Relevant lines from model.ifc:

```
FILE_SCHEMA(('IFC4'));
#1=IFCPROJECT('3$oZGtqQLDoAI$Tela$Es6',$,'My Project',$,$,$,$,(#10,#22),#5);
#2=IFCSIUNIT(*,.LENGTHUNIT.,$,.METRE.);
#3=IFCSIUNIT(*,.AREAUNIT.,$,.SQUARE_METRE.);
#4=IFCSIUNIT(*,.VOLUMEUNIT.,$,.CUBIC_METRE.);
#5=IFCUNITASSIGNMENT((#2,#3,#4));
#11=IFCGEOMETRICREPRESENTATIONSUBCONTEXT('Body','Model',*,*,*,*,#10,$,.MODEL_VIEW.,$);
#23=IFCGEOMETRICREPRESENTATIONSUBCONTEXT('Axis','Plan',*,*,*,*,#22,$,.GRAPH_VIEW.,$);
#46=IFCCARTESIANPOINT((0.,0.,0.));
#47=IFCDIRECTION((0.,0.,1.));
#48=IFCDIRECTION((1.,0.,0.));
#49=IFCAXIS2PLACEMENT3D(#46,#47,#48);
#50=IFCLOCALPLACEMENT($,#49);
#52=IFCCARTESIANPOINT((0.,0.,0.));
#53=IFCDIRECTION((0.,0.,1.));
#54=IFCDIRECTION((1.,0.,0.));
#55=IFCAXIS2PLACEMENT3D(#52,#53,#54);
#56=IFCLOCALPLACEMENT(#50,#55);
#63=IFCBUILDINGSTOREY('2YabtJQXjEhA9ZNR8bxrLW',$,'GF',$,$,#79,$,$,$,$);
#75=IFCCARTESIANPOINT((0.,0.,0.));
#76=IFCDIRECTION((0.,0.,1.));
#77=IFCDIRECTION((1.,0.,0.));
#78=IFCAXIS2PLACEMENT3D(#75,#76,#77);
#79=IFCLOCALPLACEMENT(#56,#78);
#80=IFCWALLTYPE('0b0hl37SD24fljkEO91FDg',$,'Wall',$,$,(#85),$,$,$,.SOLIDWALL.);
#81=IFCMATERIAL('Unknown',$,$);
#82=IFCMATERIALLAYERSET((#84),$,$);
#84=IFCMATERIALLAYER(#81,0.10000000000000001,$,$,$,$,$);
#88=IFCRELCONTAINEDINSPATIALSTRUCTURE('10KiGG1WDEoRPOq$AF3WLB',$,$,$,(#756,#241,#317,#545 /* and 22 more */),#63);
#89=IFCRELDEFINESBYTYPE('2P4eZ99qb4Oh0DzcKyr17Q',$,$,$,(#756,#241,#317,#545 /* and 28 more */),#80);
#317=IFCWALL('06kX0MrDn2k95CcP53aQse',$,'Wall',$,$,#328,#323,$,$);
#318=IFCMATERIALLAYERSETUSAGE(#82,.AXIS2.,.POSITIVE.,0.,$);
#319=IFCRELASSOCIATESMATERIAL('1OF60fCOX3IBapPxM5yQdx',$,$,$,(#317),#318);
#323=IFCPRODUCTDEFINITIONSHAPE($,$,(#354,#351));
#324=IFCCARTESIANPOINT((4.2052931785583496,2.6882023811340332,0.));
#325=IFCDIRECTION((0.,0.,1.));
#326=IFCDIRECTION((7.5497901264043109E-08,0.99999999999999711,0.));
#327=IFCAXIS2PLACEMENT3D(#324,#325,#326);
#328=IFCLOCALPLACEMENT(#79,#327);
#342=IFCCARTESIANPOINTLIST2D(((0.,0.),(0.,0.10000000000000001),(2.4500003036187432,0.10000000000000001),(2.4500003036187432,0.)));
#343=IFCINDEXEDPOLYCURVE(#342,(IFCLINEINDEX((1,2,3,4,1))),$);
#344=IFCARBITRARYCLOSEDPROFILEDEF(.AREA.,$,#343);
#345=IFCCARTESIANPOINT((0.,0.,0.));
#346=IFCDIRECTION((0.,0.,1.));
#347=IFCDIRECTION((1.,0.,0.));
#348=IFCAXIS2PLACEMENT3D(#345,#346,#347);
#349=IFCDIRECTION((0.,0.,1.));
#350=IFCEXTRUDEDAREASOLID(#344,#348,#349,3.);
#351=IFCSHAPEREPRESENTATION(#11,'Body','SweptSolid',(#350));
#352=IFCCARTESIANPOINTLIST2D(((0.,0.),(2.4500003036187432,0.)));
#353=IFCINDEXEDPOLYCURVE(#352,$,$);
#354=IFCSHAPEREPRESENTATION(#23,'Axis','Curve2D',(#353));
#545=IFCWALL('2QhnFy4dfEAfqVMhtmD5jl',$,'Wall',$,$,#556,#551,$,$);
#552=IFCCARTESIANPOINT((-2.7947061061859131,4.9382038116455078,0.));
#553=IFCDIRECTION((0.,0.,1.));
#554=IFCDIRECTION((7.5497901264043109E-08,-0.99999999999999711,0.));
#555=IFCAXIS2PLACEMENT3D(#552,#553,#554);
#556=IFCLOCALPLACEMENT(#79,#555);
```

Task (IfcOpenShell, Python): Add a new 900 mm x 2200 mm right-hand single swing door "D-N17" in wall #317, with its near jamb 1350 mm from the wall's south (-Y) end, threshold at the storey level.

```python
import numpy as np
import ifcopenshell
import ifcopenshell.api.feature
import ifcopenshell.api.geometry
import ifcopenshell.api.root
import ifcopenshell.api.spatial
import ifcopenshell.geom
import ifcopenshell.util.element
import ifcopenshell.util.placement
import ifcopenshell.util.representation
import ifcopenshell.util.shape
import ifcopenshell.util.unit

model = ifcopenshell.open("model.ifc")
unit_scale = ifcopenshell.util.unit.calculate_unit_scale(model)
settings = ifcopenshell.geom.settings()


def volume(element):
    """Net volume in cubic metres, openings subtracted."""
    shape = ifcopenshell.geom.create_shape(settings, element)
    return ifcopenshell.util.shape.get_volume(shape.geometry)


wall = model.by_guid("06kX0MrDn2k95CcP53aQse")
storey = ifcopenshell.util.element.get_container(wall, ifc_class="IfcBuildingStorey")
context = ifcopenshell.util.representation.get_context(model, "Model", "Body", "MODEL_VIEW")
before = volume(wall)

width, height, from_end, sill = 0.9, 2.2, 1.35, 0.0  # metres

# The wall runs along its own X axis, and the end named is its -X end.
wall_shape = ifcopenshell.geom.create_shape(settings, wall)
x, y, z = ifcopenshell.util.shape.get_vertices(wall_shape.geometry).T
start = x.min() + from_end
face, thickness = float(y.min()), float(y.max() - y.min())
wall_matrix = ifcopenshell.util.placement.get_local_placement(wall.ObjectPlacement)
level = ifcopenshell.util.placement.get_local_placement(storey.ObjectPlacement)[2, 3]


def in_wall(x, y):
    """Placement at x, y metres in the wall's axes, at sill height."""
    matrix = wall_matrix.copy()
    matrix[:, 3] = wall_matrix @ np.array([x / unit_scale, y / unit_scale, 0.0, 1.0])
    matrix[2, 3] = level + sill / unit_scale
    return matrix


# Opening: a box that overshoots both wall faces by 50 mm.
opening = ifcopenshell.api.root.create_entity(model, ifc_class="IfcOpeningElement", predefined_type="OPENING")
box = ifcopenshell.api.geometry.add_wall_representation(
    model, context=context, length=width, height=height, thickness=thickness + 0.1
)
ifcopenshell.api.geometry.assign_representation(model, product=opening, representation=box)
ifcopenshell.api.geometry.edit_object_placement(model, product=opening, matrix=in_wall(start, face - 0.05), is_si=False)
ifcopenshell.api.feature.add_feature(model, feature=opening, element=wall)

door = ifcopenshell.api.root.create_entity(model, ifc_class="IfcDoor", name="D-N17", predefined_type="DOOR")
door.OverallWidth, door.OverallHeight = width / unit_scale, height / unit_scale
door.OperationType = "SINGLE_SWING_RIGHT"
body = ifcopenshell.api.geometry.add_door_representation(
    model,
    context=context,
    overall_width=door.OverallWidth,
    overall_height=door.OverallHeight,
    operation_type="SINGLE_SWING_RIGHT",
    lining_properties={"LiningDepth": thickness / unit_scale, "ThresholdDepth": thickness / unit_scale},
)
ifcopenshell.api.geometry.assign_representation(model, product=door, representation=body)
ifcopenshell.api.spatial.assign_container(model, products=[door], relating_structure=storey)
ifcopenshell.api.feature.add_filling(model, opening=opening, element=door)

# The lining spans the wall, so the door starts at the wall face.
ifcopenshell.api.geometry.edit_object_placement(model, product=door, matrix=in_wall(start, face), is_si=False)

after = volume(wall)

print(f"wall volume {before:.3f} -> {after:.3f} m3")

model.write("model_v2.ifc")
```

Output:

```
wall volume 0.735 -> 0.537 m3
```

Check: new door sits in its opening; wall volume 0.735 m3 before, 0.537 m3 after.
